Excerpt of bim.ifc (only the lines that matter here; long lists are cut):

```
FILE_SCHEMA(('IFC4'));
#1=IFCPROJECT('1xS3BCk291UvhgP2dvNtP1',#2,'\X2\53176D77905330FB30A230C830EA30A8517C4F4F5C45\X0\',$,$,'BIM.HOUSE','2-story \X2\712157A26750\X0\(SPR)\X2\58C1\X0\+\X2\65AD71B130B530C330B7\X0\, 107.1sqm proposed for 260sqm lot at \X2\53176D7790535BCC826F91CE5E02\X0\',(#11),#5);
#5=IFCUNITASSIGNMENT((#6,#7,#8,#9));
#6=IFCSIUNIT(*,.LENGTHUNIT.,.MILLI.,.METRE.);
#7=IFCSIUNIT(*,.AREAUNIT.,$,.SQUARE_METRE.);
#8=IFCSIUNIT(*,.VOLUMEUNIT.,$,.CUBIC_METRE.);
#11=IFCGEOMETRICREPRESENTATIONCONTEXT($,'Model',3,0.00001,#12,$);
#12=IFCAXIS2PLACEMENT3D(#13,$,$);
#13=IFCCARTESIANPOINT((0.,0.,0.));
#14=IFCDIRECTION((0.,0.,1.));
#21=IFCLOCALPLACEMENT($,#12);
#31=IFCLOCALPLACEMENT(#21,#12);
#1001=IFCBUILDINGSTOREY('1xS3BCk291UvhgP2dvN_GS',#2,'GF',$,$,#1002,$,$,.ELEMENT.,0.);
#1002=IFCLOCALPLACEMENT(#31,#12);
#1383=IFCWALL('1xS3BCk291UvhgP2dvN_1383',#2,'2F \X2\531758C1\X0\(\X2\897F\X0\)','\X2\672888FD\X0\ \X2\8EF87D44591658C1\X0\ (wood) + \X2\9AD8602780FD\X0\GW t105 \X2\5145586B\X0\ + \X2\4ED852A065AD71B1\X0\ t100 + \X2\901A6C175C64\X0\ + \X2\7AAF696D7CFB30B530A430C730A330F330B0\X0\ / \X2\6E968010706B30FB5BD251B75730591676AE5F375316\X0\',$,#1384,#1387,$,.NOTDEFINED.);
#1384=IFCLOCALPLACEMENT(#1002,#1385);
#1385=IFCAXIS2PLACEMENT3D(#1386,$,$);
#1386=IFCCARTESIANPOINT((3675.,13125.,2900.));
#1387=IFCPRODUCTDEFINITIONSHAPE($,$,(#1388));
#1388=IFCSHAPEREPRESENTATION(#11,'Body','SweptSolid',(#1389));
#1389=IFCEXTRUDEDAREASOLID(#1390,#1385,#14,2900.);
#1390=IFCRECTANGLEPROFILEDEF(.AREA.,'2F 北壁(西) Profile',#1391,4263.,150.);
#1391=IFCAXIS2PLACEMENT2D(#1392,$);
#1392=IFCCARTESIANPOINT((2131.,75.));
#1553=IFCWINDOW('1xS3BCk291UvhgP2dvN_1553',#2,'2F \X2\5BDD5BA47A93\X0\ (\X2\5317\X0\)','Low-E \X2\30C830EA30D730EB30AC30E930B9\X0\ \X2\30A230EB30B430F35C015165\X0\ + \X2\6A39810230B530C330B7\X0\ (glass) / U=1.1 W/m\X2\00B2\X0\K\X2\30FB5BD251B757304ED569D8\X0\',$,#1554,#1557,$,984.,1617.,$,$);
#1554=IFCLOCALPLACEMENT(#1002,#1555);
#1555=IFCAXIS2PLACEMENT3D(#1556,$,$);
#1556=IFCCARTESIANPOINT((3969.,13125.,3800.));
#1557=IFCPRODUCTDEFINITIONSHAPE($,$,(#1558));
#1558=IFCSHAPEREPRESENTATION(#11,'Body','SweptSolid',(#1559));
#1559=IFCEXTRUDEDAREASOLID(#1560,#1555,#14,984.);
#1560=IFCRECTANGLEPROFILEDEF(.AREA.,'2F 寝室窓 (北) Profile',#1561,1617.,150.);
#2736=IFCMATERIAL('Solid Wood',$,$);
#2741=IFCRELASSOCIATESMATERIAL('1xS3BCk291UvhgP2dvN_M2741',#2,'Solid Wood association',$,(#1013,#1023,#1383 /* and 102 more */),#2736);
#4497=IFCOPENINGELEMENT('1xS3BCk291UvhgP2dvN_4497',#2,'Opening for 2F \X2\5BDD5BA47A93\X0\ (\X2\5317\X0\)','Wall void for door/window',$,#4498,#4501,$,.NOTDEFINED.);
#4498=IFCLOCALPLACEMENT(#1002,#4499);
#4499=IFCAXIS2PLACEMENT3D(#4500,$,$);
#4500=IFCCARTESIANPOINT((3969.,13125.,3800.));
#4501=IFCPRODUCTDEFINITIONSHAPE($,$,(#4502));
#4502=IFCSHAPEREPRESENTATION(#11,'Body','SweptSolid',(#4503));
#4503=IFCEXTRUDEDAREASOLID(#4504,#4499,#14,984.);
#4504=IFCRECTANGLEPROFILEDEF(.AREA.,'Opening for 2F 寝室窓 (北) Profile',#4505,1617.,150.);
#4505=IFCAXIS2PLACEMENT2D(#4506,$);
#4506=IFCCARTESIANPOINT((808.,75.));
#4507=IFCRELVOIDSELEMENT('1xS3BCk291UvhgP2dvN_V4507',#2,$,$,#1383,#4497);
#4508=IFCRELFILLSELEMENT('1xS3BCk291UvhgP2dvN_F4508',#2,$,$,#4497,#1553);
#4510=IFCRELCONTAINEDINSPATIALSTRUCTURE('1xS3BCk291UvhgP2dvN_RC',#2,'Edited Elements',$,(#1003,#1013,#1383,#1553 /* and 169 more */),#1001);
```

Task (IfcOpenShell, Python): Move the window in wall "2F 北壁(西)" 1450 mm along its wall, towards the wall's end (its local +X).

```python
import ifcopenshell
import ifcopenshell.api.geometry
import ifcopenshell.util.placement
import ifcopenshell.util.unit

model = ifcopenshell.open("bim.ifc")
unit_scale = ifcopenshell.util.unit.calculate_unit_scale(model)

window = model.by_guid("1xS3BCk291UvhgP2dvN_1553")
opening = window.FillsVoids[0].RelatingOpeningElement
wall = opening.VoidsElements[0].RelatingBuildingElement

wall_matrix = ifcopenshell.util.placement.get_local_placement(wall.ObjectPlacement)
shift = wall_matrix[:3, 0] * 1.45 / unit_scale
before = ifcopenshell.util.placement.get_local_placement(window.ObjectPlacement)[:3, 3].copy()

# The window is not placed relative to its opening, so move both.
for product in (opening, window):
    matrix = ifcopenshell.util.placement.get_local_placement(product.ObjectPlacement)
    matrix[:3, 3] += shift
    ifcopenshell.api.geometry.edit_object_placement(model, product=product, matrix=matrix, is_si=False)

after = ifcopenshell.util.placement.get_local_placement(window.ObjectPlacement)[:3, 3]
print("window moved by", (after - before).round(3) + 0.0)

model.write("bim_rev.ifc")
```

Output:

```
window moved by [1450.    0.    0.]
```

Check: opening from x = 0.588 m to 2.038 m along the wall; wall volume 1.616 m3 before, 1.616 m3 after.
